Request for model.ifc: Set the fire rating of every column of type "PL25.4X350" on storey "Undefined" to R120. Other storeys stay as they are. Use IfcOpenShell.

First a look at what the model holds.

```python
import ifcopenshell
import ifcopenshell.util.element

model = ifcopenshell.open("model.ifc")
print(model.schema)
storey = next(s for s in model.by_type("IfcBuildingStorey") if s.Name == "Undefined")
columns = [e for e in ifcopenshell.util.element.get_decomposition(storey) if e.is_a("IfcColumn")]
seen = {}
for e in columns:
    element_type = ifcopenshell.util.element.get_type(e)
    key = (element_type.Name if element_type != e and element_type else None, ifcopenshell.util.element.get_pset(e, "Pset_ColumnCommon", "FireRating"))
    seen[key] = seen.get(key, 0) + 1
for (name, value), count in sorted(seen.items(), key=str):
    print(count, "x", name, "|", value)
```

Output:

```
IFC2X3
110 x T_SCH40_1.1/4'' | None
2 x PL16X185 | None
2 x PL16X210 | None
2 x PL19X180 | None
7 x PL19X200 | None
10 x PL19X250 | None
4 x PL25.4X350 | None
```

```python
import ifcopenshell
import ifcopenshell.api.pset
import ifcopenshell.util.element

model = ifcopenshell.open("model.ifc")

storey = next(s for s in model.by_type("IfcBuildingStorey") if s.Name == "Undefined")
columns = [e for e in ifcopenshell.util.element.get_decomposition(storey) if e.is_a("IfcColumn")]

count = 0
for e in columns:
    element_type = ifcopenshell.util.element.get_type(e)
    if element_type in (None, e) or element_type.Name != "PL25.4X350":
        continue
    # add_pset returns the element's existing set when there is one.
    pset = ifcopenshell.api.pset.add_pset(model, product=e, name="Pset_ColumnCommon")
    ifcopenshell.api.pset.edit_pset(model, pset=pset, properties={"FireRating": "R120"})
    count += 1

print(count, "columns updated")

model.write("model_updated.ifc")
```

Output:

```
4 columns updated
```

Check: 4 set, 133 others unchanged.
